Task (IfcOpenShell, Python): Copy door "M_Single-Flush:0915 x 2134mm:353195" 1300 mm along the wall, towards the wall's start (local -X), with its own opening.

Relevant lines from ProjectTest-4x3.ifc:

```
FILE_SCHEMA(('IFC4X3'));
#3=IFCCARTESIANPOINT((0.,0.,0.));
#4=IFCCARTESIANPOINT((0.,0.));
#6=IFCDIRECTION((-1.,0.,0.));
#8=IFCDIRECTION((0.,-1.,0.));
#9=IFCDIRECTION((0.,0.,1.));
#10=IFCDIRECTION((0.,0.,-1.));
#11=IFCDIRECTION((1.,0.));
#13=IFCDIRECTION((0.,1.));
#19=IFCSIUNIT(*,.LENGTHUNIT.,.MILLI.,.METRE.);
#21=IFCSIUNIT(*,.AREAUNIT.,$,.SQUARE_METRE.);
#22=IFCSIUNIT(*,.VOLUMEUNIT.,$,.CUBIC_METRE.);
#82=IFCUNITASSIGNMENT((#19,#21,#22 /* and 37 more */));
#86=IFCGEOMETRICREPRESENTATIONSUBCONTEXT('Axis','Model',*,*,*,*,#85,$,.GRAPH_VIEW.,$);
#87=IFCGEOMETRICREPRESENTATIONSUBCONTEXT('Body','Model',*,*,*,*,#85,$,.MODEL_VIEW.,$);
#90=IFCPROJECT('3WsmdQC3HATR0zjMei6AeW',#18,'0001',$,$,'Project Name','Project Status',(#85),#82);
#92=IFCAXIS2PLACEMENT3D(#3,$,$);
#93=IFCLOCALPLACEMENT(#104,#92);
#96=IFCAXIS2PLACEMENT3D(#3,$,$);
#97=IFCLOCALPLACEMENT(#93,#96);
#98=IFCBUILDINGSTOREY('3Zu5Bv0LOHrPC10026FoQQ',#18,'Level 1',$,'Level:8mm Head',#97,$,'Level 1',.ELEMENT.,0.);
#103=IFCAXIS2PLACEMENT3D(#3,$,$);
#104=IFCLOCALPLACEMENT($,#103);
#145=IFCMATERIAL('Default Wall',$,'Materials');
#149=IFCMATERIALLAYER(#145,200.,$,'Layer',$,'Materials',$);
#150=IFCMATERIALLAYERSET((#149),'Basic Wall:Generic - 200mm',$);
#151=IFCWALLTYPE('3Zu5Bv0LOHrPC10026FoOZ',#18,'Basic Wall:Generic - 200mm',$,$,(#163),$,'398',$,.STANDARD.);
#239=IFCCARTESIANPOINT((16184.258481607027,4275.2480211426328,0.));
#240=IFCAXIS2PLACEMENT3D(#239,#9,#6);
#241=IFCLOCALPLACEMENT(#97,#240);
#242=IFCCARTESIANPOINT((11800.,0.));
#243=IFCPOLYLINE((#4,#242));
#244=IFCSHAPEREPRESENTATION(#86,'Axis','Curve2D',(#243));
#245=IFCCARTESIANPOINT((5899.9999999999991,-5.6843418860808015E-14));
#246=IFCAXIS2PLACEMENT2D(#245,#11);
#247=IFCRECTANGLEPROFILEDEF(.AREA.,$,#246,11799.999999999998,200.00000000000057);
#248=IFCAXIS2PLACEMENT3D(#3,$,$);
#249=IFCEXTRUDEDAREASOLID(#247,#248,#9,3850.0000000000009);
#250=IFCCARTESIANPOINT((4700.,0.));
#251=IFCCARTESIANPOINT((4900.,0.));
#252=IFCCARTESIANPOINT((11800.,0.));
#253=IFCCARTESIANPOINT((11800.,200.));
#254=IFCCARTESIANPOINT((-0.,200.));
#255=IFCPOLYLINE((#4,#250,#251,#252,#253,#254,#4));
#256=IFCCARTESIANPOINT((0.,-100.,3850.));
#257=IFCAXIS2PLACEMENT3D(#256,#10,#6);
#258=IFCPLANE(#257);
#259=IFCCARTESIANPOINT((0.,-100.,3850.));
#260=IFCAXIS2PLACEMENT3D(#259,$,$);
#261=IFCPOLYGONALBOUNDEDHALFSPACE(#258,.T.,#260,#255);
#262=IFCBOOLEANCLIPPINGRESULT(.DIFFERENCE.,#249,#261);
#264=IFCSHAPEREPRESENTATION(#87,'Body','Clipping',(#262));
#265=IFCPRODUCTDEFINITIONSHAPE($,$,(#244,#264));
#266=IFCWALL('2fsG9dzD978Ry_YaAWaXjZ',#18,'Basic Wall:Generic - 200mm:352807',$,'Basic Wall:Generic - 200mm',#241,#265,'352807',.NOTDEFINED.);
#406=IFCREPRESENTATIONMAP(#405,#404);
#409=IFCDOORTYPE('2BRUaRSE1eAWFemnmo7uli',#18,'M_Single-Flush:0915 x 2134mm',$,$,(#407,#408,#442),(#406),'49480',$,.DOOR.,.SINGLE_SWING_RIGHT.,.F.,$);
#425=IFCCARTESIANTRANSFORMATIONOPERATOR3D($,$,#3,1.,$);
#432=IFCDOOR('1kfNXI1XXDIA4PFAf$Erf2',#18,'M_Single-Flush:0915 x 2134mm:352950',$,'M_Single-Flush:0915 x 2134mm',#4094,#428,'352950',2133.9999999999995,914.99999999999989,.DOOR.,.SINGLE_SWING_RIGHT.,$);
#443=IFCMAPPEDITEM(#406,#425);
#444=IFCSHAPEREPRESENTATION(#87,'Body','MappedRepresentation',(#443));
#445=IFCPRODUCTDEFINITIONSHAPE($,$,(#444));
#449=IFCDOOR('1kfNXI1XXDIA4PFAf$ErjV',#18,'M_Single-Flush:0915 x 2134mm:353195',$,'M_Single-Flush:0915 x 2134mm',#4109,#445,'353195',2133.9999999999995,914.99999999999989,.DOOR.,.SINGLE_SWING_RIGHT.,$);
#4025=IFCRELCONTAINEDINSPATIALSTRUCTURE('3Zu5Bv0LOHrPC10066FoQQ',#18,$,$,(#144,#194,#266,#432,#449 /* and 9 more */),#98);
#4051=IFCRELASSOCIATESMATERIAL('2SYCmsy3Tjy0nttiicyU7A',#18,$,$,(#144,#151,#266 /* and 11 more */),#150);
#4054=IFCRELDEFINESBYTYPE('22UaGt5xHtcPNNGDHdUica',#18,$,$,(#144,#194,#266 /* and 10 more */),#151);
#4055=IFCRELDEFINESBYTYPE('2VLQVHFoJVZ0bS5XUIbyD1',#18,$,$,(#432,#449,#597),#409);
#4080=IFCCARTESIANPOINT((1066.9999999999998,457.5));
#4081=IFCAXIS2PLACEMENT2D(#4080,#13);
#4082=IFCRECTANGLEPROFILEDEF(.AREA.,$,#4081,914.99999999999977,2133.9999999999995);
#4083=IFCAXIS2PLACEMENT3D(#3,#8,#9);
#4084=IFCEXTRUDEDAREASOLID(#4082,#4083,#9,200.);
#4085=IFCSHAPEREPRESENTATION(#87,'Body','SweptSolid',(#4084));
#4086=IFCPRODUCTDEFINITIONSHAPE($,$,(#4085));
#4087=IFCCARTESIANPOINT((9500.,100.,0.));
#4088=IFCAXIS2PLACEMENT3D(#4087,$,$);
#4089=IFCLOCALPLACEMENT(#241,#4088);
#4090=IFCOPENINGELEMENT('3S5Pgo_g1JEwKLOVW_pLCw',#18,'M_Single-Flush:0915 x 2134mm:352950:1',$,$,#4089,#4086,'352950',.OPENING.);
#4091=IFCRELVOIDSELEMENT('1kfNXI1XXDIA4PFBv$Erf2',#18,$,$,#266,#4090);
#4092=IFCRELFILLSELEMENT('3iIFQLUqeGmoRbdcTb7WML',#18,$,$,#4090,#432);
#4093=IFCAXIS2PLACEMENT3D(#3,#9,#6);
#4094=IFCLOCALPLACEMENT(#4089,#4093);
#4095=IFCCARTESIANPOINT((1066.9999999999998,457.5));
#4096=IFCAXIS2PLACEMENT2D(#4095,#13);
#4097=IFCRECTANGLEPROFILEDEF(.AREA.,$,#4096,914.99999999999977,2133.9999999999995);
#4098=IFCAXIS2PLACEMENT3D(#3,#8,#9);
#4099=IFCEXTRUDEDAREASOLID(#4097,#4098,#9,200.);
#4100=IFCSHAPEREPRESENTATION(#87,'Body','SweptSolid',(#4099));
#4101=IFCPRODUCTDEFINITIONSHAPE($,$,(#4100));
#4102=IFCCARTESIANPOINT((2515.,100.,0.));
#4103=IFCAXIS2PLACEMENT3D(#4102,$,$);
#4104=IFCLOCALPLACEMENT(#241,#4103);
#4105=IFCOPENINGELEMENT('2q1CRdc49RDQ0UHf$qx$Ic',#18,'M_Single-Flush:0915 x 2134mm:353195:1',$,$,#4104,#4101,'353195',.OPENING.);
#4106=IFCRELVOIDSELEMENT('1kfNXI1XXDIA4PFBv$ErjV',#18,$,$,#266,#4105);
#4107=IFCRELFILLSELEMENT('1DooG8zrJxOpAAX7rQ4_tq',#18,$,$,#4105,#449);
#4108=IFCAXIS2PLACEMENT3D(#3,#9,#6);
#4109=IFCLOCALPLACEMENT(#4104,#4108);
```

```python
import ifcopenshell
import ifcopenshell.api.feature
import ifcopenshell.api.geometry
import ifcopenshell.api.root
import ifcopenshell.geom
import ifcopenshell.util.element
import ifcopenshell.util.placement
import ifcopenshell.util.shape
import ifcopenshell.util.unit

model = ifcopenshell.open("ProjectTest-4x3.ifc")
unit_scale = ifcopenshell.util.unit.calculate_unit_scale(model)
settings = ifcopenshell.geom.settings()


def volume(element):
    """Net volume in cubic metres, openings subtracted."""
    shape = ifcopenshell.geom.create_shape(settings, element)
    return ifcopenshell.util.shape.get_volume(shape.geometry)


def reuse_history(source, copy):
    """copy_class also copies each property set's owner history, people and application; keep the originals."""
    for rel in copy.IsDefinedBy:
        if rel.is_a("IfcRelDefinesByProperties") and (history := rel.RelatingPropertyDefinition.OwnerHistory):
            rel.RelatingPropertyDefinition.OwnerHistory = source.OwnerHistory
            ifcopenshell.util.element.remove_deep2(model, history)


door = model.by_id(449)
opening = door.FillsVoids[0].RelatingOpeningElement
wall = opening.VoidsElements[0].RelatingBuildingElement
before = volume(wall)
shift = ifcopenshell.util.placement.get_local_placement(wall.ObjectPlacement)[:3, 0] * -1.3 / unit_scale

# copy_class copies the void relationship, type, container and properties, but no geometry.
new_opening = ifcopenshell.api.root.copy_class(model, product=opening)
new_opening.Representation = ifcopenshell.util.element.copy_deep(
    model, opening.Representation, exclude=["IfcGeometricRepresentationContext", "IfcRepresentationMap"]
)
new_opening.Name = "M_Single-Flush:0915 x 2134mm"
new_opening.Tag = None
new_door = ifcopenshell.api.root.copy_class(model, product=door)
new_door.Representation = ifcopenshell.util.element.copy_deep(
    model, door.Representation, exclude=["IfcGeometricRepresentationContext", "IfcRepresentationMap"]
)
new_door.Name = "M_Single-Flush:0915 x 2134mm"
new_door.Tag = None
reuse_history(door, new_door)
ifcopenshell.api.feature.add_filling(model, opening=new_opening, element=new_door)

for old, new in ((opening, new_opening), (door, new_door)):
    matrix = ifcopenshell.util.placement.get_local_placement(old.ObjectPlacement)
    matrix[:3, 3] += shift
    ifcopenshell.api.geometry.edit_object_placement(model, product=new, matrix=matrix, is_si=False)

after = volume(wall)

print(f"wall volume {before:.3f} -> {after:.3f} m3")

model.write("ProjectTest-4x3_rev.ifc")
```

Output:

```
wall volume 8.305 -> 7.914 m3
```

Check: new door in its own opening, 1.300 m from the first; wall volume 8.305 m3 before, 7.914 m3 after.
